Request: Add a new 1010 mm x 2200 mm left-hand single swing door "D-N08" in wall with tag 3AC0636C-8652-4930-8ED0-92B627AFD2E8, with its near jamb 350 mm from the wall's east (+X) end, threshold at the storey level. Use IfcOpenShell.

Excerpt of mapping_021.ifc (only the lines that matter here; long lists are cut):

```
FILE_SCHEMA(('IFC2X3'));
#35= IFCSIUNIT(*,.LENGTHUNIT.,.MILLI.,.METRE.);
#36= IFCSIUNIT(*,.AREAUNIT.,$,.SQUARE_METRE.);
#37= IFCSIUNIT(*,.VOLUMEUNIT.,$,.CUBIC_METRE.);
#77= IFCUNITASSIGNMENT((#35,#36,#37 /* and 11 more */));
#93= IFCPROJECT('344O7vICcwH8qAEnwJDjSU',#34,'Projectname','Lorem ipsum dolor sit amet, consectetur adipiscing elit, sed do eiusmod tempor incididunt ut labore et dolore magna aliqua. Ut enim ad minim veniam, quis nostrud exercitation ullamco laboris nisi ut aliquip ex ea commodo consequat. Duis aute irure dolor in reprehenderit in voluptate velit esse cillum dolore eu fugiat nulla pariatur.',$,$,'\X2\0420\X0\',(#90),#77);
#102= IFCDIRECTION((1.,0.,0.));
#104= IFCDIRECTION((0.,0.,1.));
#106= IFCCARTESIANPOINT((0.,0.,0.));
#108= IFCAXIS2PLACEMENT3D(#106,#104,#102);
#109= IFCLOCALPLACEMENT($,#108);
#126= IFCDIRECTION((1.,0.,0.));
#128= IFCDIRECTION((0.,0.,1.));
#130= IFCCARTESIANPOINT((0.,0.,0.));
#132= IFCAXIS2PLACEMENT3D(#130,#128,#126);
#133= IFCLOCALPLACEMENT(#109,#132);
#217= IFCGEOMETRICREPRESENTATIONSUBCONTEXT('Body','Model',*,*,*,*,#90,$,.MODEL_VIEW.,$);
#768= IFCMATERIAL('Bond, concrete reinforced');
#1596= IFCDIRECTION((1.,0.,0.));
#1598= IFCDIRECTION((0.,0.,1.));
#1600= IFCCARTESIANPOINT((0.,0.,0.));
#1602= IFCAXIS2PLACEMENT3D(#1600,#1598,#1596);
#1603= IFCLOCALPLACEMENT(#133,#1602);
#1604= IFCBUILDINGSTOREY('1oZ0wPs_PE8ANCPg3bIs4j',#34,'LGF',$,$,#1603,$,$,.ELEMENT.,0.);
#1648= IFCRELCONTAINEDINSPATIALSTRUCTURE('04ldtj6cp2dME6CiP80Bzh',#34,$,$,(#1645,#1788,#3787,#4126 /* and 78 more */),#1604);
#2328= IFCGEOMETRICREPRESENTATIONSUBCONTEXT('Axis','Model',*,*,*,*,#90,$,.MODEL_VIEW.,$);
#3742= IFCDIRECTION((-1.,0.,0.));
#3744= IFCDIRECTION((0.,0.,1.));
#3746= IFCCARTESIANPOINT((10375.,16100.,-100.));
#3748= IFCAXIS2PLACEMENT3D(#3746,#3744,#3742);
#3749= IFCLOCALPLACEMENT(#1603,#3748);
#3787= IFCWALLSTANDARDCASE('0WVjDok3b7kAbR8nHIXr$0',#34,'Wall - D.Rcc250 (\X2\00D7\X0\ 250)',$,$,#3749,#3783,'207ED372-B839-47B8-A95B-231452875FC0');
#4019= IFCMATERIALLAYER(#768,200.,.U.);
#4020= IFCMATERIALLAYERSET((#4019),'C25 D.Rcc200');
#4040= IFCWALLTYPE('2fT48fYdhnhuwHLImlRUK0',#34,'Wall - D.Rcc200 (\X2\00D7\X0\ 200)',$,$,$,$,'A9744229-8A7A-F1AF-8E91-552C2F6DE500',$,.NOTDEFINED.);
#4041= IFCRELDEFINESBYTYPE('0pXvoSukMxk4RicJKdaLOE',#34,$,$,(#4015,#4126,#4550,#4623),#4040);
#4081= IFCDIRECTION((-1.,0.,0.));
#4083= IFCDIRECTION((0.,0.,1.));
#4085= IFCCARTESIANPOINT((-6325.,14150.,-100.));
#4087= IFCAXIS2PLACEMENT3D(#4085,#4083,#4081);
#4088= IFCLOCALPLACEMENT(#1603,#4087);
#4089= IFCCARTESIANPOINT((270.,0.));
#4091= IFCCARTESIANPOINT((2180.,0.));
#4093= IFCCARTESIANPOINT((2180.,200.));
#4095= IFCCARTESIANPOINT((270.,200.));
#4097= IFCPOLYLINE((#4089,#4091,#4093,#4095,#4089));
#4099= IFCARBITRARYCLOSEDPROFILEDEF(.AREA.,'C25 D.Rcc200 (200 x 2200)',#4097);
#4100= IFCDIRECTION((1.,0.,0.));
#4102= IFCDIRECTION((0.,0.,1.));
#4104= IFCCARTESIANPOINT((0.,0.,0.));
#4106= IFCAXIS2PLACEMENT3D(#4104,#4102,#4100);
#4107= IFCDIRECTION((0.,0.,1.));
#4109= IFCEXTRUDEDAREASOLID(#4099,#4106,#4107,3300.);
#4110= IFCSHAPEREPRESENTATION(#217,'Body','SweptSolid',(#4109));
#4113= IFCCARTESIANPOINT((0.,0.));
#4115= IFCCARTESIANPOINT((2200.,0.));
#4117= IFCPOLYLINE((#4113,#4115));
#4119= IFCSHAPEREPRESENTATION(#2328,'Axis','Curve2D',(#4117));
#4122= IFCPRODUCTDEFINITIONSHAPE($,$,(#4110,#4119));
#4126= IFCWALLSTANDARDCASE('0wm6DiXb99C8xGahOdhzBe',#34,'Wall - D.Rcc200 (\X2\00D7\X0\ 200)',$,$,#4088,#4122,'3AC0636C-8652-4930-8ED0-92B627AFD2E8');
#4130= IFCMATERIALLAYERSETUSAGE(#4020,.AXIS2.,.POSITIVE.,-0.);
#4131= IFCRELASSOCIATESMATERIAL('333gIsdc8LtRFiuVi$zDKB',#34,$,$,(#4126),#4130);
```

```python
import numpy as np
import ifcopenshell
import ifcopenshell.api.feature
import ifcopenshell.api.geometry
import ifcopenshell.api.root
import ifcopenshell.api.spatial
import ifcopenshell.api.type
import ifcopenshell.geom
import ifcopenshell.util.element
import ifcopenshell.util.placement
import ifcopenshell.util.representation
import ifcopenshell.util.shape
import ifcopenshell.util.unit

model = ifcopenshell.open("mapping_021.ifc")
unit_scale = ifcopenshell.util.unit.calculate_unit_scale(model)
settings = ifcopenshell.geom.settings()


def volume(element):
    """Net volume in cubic metres, openings subtracted."""
    shape = ifcopenshell.geom.create_shape(settings, element)
    return ifcopenshell.util.shape.get_volume(shape.geometry)


wall = model.by_guid("0wm6DiXb99C8xGahOdhzBe")
storey = ifcopenshell.util.element.get_container(wall, ifc_class="IfcBuildingStorey")
context = ifcopenshell.util.representation.get_context(model, "Model", "Body", "MODEL_VIEW")
before = volume(wall)

width, height, from_end, sill = 1.01, 2.2, 0.35, 0.0  # metres

# The wall runs along its own X axis, and the end named is its -X end.
wall_shape = ifcopenshell.geom.create_shape(settings, wall)
x, y, z = ifcopenshell.util.shape.get_vertices(wall_shape.geometry).T
start = x.min() + from_end
face, thickness = float(y.min()), float(y.max() - y.min())
wall_matrix = ifcopenshell.util.placement.get_local_placement(wall.ObjectPlacement)
level = ifcopenshell.util.placement.get_local_placement(storey.ObjectPlacement)[2, 3]


def in_wall(x, y):
    """Placement at x, y metres in the wall's axes, at sill height."""
    matrix = wall_matrix.copy()
    matrix[:, 3] = wall_matrix @ np.array([x / unit_scale, y / unit_scale, 0.0, 1.0])
    matrix[2, 3] = level + sill / unit_scale
    return matrix


# Opening: a box that overshoots both wall faces by 50 mm.
opening = ifcopenshell.api.root.create_entity(model, ifc_class="IfcOpeningElement")
box = ifcopenshell.api.geometry.add_wall_representation(
    model, context=context, length=width, height=height, thickness=thickness + 0.1
)
ifcopenshell.api.geometry.assign_representation(model, product=opening, representation=box)
ifcopenshell.api.geometry.edit_object_placement(model, product=opening, matrix=in_wall(start, face - 0.05), is_si=False)
ifcopenshell.api.feature.add_feature(model, feature=opening, element=wall)

door = ifcopenshell.api.root.create_entity(model, ifc_class="IfcDoor", name="D-N08")
door.OverallWidth, door.OverallHeight = width / unit_scale, height / unit_scale
body = ifcopenshell.api.geometry.add_door_representation(
    model,
    context=context,
    overall_width=door.OverallWidth,
    overall_height=door.OverallHeight,
    operation_type="SINGLE_SWING_LEFT",
    lining_properties={"LiningDepth": thickness / unit_scale, "ThresholdDepth": thickness / unit_scale},
)
ifcopenshell.api.geometry.assign_representation(model, product=door, representation=body)
ifcopenshell.api.spatial.assign_container(model, products=[door], relating_structure=storey)
fills = ifcopenshell.api.feature.add_filling(model, opening=opening, element=door)
fills.OwnerHistory = door.OwnerHistory  # required in IFC2X3

# IFC2X3 keeps the operation on the door style.
style = ifcopenshell.api.root.create_entity(model, ifc_class="IfcDoorStyle", name="D-N08")
style.OperationType, style.ConstructionType = "SINGLE_SWING_LEFT", "NOTDEFINED"
style.ParameterTakesPrecedence = style.Sizeable = False
ifcopenshell.api.type.assign_type(model, related_objects=[door], relating_type=style)

# The lining spans the wall, so the door starts at the wall face.
ifcopenshell.api.geometry.edit_object_placement(model, product=door, matrix=in_wall(start, face), is_si=False)

after = volume(wall)

print(f"wall volume {before:.3f} -> {after:.3f} m3")

model.write("mapping_021_updated.ifc")
```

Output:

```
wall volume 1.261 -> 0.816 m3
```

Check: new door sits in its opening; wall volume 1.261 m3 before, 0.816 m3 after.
